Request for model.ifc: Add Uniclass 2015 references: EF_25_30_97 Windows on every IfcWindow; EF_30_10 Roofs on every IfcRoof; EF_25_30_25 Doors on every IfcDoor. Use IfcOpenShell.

First a look at what the model holds.

```python
import ifcopenshell

model = ifcopenshell.open("model.ifc")
print(model.schema)
print("classifications:", [c.Name for c in model.by_type("IfcClassification")])
for ifc_class in ("IfcDoor", "IfcRoof", "IfcStair", "IfcWall", "IfcWindow"):
    print(ifc_class, len(model.by_type(ifc_class)))
```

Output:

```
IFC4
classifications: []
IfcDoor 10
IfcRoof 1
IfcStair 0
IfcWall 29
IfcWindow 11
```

```python
import ifcopenshell
import ifcopenshell.api.classification

model = ifcopenshell.open("model.ifc")

system = ifcopenshell.api.classification.add_classification(model, classification="Uniclass 2015")

codes = {
    "IfcWindow": ("EF_25_30_97", "Windows"),
    "IfcRoof": ("EF_30_10", "Roofs"),
    "IfcDoor": ("EF_25_30_25", "Doors"),
}
for ifc_class, (code, name) in codes.items():
    products = model.by_type(ifc_class)
    ifcopenshell.api.classification.add_reference(
        model, products=products, classification=system, identification=code, name=name
    )
    print(code, len(products))

model.write("model-out.ifc")
```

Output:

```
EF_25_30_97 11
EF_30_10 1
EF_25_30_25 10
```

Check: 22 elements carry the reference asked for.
